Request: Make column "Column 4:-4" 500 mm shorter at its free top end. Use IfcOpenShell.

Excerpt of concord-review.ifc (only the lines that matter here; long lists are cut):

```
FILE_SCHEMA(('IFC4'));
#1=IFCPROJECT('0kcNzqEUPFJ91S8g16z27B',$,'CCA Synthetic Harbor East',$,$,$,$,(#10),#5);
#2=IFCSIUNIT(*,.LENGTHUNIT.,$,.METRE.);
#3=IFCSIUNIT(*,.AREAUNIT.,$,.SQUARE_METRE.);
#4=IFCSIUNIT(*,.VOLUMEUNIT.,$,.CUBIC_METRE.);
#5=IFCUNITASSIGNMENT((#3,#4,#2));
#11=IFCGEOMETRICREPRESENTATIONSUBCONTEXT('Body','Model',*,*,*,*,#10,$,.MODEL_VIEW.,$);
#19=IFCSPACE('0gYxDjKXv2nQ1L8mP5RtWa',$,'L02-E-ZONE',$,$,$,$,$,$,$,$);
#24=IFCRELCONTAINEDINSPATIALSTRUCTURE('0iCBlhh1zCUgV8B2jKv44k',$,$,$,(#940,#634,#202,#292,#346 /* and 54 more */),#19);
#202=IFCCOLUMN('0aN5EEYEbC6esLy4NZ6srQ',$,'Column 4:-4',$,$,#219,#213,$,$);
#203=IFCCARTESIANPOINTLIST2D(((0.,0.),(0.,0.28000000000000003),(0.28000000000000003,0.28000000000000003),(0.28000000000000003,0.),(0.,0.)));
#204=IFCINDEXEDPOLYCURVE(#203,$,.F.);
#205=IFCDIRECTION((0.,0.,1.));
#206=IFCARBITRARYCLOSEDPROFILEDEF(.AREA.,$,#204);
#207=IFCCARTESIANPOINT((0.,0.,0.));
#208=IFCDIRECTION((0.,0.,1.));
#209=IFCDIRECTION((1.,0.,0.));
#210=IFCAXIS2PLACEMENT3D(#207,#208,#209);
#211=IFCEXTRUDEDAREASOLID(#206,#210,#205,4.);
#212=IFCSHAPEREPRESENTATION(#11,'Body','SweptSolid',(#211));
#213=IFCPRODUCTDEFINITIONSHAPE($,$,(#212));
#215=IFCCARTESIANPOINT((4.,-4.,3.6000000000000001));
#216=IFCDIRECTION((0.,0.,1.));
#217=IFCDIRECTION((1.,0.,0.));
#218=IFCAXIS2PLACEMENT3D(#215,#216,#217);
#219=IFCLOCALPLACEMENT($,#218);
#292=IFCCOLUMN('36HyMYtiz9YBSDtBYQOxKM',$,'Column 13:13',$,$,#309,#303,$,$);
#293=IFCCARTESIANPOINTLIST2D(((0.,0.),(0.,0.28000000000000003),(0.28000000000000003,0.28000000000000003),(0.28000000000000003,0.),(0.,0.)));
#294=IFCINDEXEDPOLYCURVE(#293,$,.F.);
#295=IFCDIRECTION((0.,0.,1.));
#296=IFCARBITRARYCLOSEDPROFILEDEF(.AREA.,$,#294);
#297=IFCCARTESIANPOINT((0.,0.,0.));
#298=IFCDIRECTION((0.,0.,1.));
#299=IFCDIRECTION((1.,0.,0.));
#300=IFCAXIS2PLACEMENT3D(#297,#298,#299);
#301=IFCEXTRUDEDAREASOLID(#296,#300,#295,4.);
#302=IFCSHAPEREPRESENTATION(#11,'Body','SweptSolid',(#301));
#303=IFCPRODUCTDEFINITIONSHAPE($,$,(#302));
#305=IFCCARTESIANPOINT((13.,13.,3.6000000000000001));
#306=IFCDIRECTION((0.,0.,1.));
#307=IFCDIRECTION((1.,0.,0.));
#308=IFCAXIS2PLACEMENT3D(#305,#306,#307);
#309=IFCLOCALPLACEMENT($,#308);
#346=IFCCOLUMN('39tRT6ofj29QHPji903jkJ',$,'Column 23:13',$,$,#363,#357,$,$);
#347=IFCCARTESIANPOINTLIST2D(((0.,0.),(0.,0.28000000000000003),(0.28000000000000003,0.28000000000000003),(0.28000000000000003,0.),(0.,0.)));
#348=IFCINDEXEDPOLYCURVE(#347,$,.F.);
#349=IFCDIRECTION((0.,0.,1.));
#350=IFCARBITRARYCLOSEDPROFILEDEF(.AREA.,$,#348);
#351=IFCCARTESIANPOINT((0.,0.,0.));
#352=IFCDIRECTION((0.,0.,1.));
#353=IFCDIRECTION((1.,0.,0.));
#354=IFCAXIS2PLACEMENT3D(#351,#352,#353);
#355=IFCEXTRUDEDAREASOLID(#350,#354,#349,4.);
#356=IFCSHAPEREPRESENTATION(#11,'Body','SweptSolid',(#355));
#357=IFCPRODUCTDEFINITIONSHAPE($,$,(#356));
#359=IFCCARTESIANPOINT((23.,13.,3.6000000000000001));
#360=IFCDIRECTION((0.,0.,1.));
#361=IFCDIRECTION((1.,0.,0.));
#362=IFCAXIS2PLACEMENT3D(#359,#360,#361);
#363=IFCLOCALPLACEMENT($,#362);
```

```python
import ifcopenshell
import ifcopenshell.util.representation
import ifcopenshell.util.unit

model = ifcopenshell.open("concord-review.ifc")
unit_scale = ifcopenshell.util.unit.calculate_unit_scale(model)

member = model.by_guid("0aN5EEYEbC6esLy4NZ6srQ")
change = -0.5 / unit_scale

# The extrusion runs towards the end named, so only its depth changes.
body = ifcopenshell.util.representation.get_representation(member, "Model", "Body")
solid = body.Items[0]
old_length = solid.Depth
solid.Depth += change

print(f"length {old_length:g} -> {solid.Depth:g}")

model.write("concord-review_edited.ifc")
```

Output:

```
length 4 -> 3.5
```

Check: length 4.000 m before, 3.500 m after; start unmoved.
